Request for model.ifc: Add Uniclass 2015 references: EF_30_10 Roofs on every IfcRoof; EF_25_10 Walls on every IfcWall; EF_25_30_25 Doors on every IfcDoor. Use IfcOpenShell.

First a look at what the model holds.

```python
import ifcopenshell

model = ifcopenshell.open("model.ifc")
print(model.schema)
print("classifications:", [c.Name for c in model.by_type("IfcClassification")])
for ifc_class in ("IfcDoor", "IfcRoof", "IfcStair", "IfcWall", "IfcWindow"):
    print(ifc_class, len(model.by_type(ifc_class)))
```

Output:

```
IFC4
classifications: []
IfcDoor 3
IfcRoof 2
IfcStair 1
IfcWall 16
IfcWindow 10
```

```python
import ifcopenshell
import ifcopenshell.api.classification

model = ifcopenshell.open("model.ifc")

system = ifcopenshell.api.classification.add_classification(model, classification="Uniclass 2015")

codes = {
    "IfcRoof": ("EF_30_10", "Roofs"),
    "IfcWall": ("EF_25_10", "Walls"),
    "IfcDoor": ("EF_25_30_25", "Doors"),
}
for ifc_class, (code, name) in codes.items():
    products = model.by_type(ifc_class)
    ifcopenshell.api.classification.add_reference(
        model, products=products, classification=system, identification=code, name=name
    )
    print(code, len(products))

model.write("model-out.ifc")
```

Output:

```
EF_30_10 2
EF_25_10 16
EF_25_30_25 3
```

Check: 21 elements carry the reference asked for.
